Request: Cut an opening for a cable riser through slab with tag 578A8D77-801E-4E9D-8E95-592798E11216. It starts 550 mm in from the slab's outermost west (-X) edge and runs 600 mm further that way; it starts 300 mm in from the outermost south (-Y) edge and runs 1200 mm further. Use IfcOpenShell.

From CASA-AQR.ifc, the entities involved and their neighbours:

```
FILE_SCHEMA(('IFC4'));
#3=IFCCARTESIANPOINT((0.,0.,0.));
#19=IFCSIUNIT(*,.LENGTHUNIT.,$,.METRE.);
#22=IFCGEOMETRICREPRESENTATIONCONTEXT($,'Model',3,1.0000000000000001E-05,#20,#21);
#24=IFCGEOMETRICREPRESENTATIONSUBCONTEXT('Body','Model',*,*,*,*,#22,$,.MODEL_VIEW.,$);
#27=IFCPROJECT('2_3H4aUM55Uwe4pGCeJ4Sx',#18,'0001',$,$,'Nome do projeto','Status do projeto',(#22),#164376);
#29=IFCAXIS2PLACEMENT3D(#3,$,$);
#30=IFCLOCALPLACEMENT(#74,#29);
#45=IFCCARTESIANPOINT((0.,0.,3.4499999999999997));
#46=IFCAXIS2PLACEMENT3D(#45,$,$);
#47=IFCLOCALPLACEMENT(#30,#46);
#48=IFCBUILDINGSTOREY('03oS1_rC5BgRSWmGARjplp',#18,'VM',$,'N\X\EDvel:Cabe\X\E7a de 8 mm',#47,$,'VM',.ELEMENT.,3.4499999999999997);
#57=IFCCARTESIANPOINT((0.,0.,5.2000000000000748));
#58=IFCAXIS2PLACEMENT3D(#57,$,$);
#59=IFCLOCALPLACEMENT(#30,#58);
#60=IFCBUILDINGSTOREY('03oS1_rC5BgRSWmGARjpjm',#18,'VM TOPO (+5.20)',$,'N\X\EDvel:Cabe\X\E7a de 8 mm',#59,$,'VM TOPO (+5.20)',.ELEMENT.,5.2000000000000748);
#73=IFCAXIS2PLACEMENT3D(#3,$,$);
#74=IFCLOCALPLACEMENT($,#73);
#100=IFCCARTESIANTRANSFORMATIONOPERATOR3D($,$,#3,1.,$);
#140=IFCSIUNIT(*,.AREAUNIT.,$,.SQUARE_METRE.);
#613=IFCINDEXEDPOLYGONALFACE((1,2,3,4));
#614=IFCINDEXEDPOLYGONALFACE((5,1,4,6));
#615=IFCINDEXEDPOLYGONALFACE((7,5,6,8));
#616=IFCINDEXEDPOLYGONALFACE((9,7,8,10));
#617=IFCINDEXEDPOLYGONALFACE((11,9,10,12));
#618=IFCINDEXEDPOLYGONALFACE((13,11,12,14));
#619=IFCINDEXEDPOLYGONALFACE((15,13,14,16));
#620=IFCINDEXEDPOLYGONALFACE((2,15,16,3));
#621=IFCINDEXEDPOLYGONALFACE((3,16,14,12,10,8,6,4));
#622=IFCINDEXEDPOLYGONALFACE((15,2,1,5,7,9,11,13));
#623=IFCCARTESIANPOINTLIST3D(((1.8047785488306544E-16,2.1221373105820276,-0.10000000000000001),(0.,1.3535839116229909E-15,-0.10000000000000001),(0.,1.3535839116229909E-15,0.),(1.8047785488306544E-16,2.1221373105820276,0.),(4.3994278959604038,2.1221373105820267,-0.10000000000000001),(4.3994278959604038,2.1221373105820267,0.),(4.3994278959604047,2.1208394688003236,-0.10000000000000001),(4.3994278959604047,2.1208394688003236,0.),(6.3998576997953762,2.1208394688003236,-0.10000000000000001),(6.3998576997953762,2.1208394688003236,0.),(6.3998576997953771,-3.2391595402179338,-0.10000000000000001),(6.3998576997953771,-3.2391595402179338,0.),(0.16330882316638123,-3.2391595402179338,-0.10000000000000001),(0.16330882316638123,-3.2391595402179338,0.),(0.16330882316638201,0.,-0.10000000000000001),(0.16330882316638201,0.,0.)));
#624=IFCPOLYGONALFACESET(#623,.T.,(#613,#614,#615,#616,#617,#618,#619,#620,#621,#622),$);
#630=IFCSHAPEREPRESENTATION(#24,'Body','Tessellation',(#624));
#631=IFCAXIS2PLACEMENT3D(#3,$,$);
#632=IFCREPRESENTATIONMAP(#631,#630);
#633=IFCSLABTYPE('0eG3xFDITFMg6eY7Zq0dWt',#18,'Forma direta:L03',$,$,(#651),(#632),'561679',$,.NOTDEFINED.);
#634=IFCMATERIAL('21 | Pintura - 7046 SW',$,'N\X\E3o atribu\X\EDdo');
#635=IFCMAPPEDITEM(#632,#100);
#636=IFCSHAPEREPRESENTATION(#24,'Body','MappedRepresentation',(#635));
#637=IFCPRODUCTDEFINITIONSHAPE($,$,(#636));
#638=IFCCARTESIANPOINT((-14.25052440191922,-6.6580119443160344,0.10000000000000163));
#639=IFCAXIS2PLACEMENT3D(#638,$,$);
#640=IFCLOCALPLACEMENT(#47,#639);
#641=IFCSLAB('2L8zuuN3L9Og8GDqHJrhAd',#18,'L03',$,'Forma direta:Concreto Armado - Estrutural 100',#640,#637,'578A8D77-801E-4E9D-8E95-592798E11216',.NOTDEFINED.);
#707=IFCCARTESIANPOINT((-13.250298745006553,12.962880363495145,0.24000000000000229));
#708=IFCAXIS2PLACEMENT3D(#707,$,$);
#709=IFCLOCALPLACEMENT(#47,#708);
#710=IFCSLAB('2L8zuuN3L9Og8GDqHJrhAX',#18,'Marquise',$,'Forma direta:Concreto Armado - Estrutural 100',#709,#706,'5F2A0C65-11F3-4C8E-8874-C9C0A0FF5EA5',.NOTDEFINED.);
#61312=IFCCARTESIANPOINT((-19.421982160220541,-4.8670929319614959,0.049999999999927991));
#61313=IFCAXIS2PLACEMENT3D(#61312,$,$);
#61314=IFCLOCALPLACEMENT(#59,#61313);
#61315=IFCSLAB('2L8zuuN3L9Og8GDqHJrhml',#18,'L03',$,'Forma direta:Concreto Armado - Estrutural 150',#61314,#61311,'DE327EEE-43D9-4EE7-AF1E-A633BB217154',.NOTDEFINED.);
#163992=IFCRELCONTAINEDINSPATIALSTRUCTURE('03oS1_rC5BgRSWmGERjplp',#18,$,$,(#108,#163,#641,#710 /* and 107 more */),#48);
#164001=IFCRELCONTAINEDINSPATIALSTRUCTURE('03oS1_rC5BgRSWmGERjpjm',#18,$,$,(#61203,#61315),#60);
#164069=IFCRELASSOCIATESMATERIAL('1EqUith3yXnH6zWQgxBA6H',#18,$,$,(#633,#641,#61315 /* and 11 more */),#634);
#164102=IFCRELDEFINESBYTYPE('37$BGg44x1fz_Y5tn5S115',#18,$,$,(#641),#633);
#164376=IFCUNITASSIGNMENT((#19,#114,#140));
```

```python
import numpy as np
import ifcopenshell
import ifcopenshell.api.feature
import ifcopenshell.api.geometry
import ifcopenshell.api.root
import ifcopenshell.geom
import ifcopenshell.util.placement
import ifcopenshell.util.representation
import ifcopenshell.util.shape
import ifcopenshell.util.unit

model = ifcopenshell.open("CASA-AQR.ifc")
unit_scale = ifcopenshell.util.unit.calculate_unit_scale(model)
settings = ifcopenshell.geom.settings()


def volume(element):
    """Net volume in cubic metres, openings subtracted."""
    shape = ifcopenshell.geom.create_shape(settings, element)
    return ifcopenshell.util.shape.get_volume(shape.geometry)


slab = model.by_guid("2L8zuuN3L9Og8GDqHJrhAd")
before = volume(slab)

# Extent in the slab's own axes, in metres. The edges named are its -X and -Y sides.
slab_shape = ifcopenshell.geom.create_shape(settings, slab)
vertices = ifcopenshell.util.shape.get_vertices(slab_shape.geometry)
x_min, y_min, bottom = vertices.min(axis=0)
top = vertices[:, 2].max()

opening = ifcopenshell.api.root.create_entity(model, ifc_class="IfcOpeningElement", name="Cable riser opening", predefined_type="OPENING")
context = ifcopenshell.util.representation.get_context(model, "Model", "Body", "MODEL_VIEW")
width, depth = 0.6, 1.2
outline = [(0.0, 0.0), (width, 0.0), (width, depth), (0.0, depth), (0.0, 0.0)]
# Overshoot both faces by 50 mm so the cut is clean.
shape = ifcopenshell.api.geometry.add_slab_representation(
    model, context=context, depth=top - bottom + 0.1, polyline=outline
)
ifcopenshell.api.geometry.assign_representation(model, product=opening, representation=shape)

matrix = ifcopenshell.util.placement.get_local_placement(slab.ObjectPlacement)
matrix[:, 3] = matrix @ np.append(np.array([x_min + 0.55, y_min + 0.3, bottom - 0.05]) / unit_scale, 1.0)
ifcopenshell.api.geometry.edit_object_placement(model, product=opening, matrix=matrix, is_si=False)
ifcopenshell.api.feature.add_feature(model, feature=opening, element=slab)

after = volume(slab)

print(f"slab volume {before:.3f} -> {after:.3f} m3")

model.write("CASA-AQR-out.ifc")
```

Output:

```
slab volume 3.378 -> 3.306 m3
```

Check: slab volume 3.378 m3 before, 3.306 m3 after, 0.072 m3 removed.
